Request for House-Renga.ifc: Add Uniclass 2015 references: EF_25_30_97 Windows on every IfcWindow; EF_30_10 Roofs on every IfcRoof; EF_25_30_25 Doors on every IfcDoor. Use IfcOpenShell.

First a look at what the model holds.

```python
import ifcopenshell

model = ifcopenshell.open("House-Renga.ifc")
print(model.schema)
print("classifications:", [c.Name for c in model.by_type("IfcClassification")])
for ifc_class in ("IfcDoor", "IfcRoof", "IfcStair", "IfcWall", "IfcWindow"):
    print(ifc_class, len(model.by_type(ifc_class)))
```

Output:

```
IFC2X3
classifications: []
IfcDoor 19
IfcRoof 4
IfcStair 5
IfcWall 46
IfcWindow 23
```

```python
import ifcopenshell
import ifcopenshell.api.classification

model = ifcopenshell.open("House-Renga.ifc")

# IFC2X3 requires Source and Edition and has no link from the project to the system.
system = model.create_entity("IfcClassification", Source="NBS", Edition="2015", Name="Uniclass 2015")

codes = {
    "IfcWindow": ("EF_25_30_97", "Windows"),
    "IfcRoof": ("EF_30_10", "Roofs"),
    "IfcDoor": ("EF_25_30_25", "Doors"),
}
for ifc_class, (code, name) in codes.items():
    products = model.by_type(ifc_class)
    ifcopenshell.api.classification.add_reference(
        model, products=products, classification=system, identification=code, name=name
    )
    print(code, len(products))

model.write("House-Renga-out.ifc")
```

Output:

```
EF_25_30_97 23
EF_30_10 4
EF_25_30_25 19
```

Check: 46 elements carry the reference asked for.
